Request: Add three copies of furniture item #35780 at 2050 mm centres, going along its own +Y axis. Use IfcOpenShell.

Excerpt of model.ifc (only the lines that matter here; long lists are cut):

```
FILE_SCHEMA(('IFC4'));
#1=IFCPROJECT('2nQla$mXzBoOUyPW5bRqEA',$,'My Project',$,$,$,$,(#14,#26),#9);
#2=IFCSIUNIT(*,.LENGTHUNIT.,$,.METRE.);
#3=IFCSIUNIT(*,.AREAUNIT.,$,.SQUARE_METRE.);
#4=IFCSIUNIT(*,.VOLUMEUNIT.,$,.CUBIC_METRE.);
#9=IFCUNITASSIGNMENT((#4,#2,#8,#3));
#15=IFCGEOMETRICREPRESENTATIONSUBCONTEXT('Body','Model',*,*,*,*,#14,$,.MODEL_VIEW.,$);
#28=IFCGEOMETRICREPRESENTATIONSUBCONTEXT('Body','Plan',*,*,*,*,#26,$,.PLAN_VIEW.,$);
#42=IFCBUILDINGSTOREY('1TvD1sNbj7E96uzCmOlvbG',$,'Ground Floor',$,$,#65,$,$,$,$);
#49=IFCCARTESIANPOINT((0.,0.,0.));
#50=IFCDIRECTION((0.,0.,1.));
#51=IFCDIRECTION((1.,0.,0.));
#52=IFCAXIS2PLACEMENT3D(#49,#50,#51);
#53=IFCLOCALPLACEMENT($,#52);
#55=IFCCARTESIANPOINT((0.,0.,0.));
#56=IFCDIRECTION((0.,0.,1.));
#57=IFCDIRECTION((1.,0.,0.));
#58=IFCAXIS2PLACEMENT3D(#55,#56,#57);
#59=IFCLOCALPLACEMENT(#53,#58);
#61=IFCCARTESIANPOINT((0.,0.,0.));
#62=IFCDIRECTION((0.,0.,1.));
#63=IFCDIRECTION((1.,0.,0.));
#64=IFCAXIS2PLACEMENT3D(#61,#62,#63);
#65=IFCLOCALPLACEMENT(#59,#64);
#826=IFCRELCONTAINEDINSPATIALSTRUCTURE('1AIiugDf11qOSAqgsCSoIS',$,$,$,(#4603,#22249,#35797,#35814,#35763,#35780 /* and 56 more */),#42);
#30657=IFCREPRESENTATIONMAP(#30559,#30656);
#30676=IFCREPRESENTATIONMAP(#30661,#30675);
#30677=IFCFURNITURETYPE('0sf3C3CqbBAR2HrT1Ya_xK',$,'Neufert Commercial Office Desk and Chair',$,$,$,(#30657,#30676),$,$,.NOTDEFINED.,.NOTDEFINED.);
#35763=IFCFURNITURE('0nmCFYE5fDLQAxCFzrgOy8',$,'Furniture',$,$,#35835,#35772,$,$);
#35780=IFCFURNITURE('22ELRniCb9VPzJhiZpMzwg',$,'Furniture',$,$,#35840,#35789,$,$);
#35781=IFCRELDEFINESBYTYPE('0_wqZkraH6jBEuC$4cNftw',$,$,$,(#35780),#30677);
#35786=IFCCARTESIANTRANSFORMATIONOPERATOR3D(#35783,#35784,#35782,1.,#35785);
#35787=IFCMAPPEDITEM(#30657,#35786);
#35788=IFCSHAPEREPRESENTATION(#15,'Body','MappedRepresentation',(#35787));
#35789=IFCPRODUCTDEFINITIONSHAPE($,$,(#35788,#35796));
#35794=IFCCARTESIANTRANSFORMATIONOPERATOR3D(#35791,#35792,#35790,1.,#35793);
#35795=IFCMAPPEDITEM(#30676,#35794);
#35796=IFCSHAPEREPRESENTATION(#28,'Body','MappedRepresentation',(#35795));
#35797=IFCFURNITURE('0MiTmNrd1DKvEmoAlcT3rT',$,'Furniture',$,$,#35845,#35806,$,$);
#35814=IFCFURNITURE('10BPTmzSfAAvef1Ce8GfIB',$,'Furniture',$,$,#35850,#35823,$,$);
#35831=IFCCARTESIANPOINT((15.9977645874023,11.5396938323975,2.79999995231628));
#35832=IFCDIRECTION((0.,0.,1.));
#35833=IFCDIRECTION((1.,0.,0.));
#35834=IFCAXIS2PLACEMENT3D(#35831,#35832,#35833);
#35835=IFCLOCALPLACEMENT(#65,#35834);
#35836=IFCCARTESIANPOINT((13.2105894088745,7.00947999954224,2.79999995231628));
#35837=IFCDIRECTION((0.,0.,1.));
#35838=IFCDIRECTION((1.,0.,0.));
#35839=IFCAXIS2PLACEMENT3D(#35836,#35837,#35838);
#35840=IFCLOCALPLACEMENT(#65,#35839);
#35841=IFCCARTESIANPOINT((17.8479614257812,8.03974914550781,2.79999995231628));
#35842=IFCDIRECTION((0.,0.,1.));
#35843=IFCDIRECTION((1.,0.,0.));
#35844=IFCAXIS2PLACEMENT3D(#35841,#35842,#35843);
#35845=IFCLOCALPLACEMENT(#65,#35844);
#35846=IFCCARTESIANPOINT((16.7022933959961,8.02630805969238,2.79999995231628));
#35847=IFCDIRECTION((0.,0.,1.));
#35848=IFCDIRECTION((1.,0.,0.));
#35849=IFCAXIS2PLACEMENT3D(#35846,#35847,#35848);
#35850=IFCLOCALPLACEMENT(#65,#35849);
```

```python
import ifcopenshell
import ifcopenshell.api.geometry
import ifcopenshell.api.root
import ifcopenshell.util.element
import ifcopenshell.util.placement

model = ifcopenshell.open("model.ifc")

source = model.by_guid("22ELRniCb9VPzJhiZpMzwg")
base = ifcopenshell.util.placement.get_local_placement(source.ObjectPlacement)
step = base[:3, 1] * 2.05

for i in range(1, 4):
    copy = ifcopenshell.api.root.copy_class(model, product=source)
    copy.Representation = ifcopenshell.util.element.copy_deep(
        model, source.Representation, exclude=["IfcGeometricRepresentationContext", "IfcRepresentationMap"]
    )
    matrix = base.copy()
    matrix[:3, 3] += i * step
    print("added at", matrix[:3, 3].round(3) + 0.0)
    ifcopenshell.api.geometry.edit_object_placement(model, product=copy, matrix=matrix, is_si=False)

model.write("model_updated.ifc")
```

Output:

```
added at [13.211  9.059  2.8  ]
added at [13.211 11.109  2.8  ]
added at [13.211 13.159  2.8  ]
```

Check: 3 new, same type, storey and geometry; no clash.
